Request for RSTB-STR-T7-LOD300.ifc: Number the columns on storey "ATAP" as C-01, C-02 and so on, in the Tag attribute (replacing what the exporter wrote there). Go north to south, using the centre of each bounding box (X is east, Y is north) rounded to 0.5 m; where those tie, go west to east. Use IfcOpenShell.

First a look at what the model holds.

```python
import ifcopenshell
import ifcopenshell.util.element
import ifcopenshell.util.placement

model = ifcopenshell.open("RSTB-STR-T7-LOD300.ifc")
print(model.schema)
storey = next(s for s in model.by_type("IfcBuildingStorey") if s.Name == "ATAP")
columns = [e for e in ifcopenshell.util.element.get_decomposition(storey) if e.is_a("IfcColumn")]
for e in sorted(columns, key=lambda e: e.id()):
    origin = ifcopenshell.util.placement.get_local_placement(e.ObjectPlacement)[:3, 3]
    print(e.id(), e.Tag, e.Name, origin.round(2) + 0.0, sep=" | ")
```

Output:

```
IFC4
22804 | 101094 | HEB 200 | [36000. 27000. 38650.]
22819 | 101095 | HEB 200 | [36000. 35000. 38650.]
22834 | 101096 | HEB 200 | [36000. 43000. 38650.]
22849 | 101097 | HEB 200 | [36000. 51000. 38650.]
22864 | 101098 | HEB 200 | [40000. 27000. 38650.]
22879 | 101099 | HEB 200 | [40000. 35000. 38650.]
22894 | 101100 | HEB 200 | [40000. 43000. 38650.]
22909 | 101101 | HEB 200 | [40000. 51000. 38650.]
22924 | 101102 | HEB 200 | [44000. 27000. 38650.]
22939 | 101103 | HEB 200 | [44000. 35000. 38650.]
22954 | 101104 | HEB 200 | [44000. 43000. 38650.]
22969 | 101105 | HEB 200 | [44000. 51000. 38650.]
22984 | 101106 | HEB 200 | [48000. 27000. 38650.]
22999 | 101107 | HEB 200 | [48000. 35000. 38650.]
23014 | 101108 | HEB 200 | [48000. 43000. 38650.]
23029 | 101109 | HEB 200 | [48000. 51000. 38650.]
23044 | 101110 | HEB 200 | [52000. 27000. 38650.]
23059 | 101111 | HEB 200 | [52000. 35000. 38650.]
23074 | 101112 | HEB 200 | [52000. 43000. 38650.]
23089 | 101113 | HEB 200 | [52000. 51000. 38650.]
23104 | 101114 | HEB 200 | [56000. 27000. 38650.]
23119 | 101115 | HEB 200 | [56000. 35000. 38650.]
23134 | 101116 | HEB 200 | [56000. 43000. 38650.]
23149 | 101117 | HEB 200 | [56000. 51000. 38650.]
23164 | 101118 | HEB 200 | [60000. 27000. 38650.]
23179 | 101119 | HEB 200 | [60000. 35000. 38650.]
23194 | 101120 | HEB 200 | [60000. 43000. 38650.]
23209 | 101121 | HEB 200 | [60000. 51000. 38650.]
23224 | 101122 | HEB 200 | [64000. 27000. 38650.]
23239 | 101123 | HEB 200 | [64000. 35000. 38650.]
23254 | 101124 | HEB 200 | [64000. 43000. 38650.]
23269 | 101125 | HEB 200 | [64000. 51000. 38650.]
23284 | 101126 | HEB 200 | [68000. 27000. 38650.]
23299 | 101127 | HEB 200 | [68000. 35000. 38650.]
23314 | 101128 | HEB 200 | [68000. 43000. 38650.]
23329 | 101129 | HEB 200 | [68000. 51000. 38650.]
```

```python
import ifcopenshell
import ifcopenshell.geom
import ifcopenshell.util.element
import ifcopenshell.util.shape

model = ifcopenshell.open("RSTB-STR-T7-LOD300.ifc")
settings = ifcopenshell.geom.settings()
settings.set("use-world-coords", True)


def centre(element):
    shape = ifcopenshell.geom.create_shape(settings, element)
    return ifcopenshell.util.shape.get_bbox_centroid(shape.geometry)


storey = next(s for s in model.by_type("IfcBuildingStorey") if s.Name == "ATAP")
columns = [e for e in ifcopenshell.util.element.get_decomposition(storey) if e.is_a("IfcColumn")]

# Insertion points can sit at a corner or the storey origin, so sort by the geometry (in metres).
centres = {e: centre(e) for e in columns}
columns.sort(key=lambda e: (-round(centres[e][1] / 0.5), centres[e][0]))

for i, e in enumerate(columns, start=1):
    number = f"C-{i:02d}"
    e.Tag = number
    print(e.id(), number)

model.write("RSTB-STR-T7-LOD300_v2.ifc")
```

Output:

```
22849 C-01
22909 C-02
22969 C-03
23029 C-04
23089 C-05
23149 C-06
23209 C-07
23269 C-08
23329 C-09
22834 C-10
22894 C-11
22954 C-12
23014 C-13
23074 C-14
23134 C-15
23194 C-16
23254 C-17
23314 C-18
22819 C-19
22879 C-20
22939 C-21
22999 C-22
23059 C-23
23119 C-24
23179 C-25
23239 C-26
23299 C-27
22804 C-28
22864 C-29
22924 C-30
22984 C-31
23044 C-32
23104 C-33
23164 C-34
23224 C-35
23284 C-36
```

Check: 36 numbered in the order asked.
